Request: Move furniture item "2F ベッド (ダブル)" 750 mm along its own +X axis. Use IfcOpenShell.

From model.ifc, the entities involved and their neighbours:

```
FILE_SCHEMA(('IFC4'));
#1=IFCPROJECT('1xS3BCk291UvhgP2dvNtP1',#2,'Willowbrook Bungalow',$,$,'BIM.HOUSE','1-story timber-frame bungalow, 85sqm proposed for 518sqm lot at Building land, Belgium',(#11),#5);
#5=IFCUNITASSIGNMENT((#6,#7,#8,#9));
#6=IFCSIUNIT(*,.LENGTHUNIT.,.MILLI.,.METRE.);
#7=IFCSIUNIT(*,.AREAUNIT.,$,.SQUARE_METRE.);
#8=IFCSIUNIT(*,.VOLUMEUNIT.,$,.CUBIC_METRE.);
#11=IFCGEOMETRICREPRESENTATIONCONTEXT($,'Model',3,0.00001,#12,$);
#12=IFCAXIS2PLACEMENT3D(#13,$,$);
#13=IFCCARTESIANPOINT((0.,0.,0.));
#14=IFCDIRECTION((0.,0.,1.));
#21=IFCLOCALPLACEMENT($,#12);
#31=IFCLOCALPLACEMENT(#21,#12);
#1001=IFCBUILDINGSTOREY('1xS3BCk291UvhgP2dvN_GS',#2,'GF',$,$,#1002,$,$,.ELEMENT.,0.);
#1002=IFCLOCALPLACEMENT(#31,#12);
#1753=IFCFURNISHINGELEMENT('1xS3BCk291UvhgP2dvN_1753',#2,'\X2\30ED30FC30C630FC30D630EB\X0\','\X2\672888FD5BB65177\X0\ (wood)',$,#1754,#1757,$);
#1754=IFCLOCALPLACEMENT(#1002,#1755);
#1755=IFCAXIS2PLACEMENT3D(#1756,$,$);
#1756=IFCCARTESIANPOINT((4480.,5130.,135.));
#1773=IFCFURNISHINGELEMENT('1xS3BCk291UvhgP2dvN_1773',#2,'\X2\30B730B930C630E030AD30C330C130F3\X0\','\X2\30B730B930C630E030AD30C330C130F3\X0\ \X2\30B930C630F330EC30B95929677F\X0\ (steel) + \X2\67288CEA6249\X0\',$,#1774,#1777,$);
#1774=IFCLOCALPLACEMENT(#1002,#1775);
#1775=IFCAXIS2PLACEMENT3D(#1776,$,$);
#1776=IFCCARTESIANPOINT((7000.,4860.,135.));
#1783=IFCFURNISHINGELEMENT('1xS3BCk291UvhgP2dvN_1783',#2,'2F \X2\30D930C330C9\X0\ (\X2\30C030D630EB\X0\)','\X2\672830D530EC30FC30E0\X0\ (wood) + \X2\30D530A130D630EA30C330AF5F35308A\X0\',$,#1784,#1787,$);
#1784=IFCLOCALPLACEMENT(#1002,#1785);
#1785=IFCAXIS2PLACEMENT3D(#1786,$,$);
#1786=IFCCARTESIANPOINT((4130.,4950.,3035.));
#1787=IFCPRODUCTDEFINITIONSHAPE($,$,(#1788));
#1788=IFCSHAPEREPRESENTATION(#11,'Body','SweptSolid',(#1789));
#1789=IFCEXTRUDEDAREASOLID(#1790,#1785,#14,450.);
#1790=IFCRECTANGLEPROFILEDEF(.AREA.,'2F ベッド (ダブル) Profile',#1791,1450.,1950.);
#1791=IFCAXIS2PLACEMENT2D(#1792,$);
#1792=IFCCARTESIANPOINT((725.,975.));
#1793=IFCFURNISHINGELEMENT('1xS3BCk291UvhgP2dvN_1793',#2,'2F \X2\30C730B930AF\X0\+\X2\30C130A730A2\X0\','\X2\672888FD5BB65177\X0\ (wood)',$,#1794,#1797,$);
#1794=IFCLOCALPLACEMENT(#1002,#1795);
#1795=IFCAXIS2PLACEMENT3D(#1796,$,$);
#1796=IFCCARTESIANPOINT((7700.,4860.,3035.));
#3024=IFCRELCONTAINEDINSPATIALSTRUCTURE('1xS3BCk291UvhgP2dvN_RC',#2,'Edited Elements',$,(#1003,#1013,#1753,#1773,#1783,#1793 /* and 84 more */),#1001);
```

```python
import ifcopenshell
import ifcopenshell.api.geometry
import ifcopenshell.util.placement

model = ifcopenshell.open("model.ifc")

item = model.by_guid("1xS3BCk291UvhgP2dvN_1783")
matrix = ifcopenshell.util.placement.get_local_placement(item.ObjectPlacement)
matrix[:3, 3] += matrix[:3, 0] * 750.0
ifcopenshell.api.geometry.edit_object_placement(model, product=item, matrix=matrix, is_si=False)

print(ifcopenshell.util.placement.get_local_placement(item.ObjectPlacement).round(3) + 0.0)

model.write("model_rev.ifc")
```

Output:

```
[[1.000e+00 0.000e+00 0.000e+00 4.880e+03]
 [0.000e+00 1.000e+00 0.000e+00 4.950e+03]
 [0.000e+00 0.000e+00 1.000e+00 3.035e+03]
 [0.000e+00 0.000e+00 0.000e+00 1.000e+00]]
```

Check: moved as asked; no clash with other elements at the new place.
